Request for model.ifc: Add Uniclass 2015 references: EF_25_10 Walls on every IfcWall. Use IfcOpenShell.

First a look at what the model holds.

```python
import ifcopenshell

model = ifcopenshell.open("model.ifc")
print(model.schema)
print("classifications:", [c.Name for c in model.by_type("IfcClassification")])
for ifc_class in ("IfcDoor", "IfcRoof", "IfcStair", "IfcWall", "IfcWindow"):
    print(ifc_class, len(model.by_type(ifc_class)))
```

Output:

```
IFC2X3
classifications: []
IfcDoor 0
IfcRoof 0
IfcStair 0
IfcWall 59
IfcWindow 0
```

```python
import ifcopenshell
import ifcopenshell.api.classification

model = ifcopenshell.open("model.ifc")

# IFC2X3 requires Source and Edition and has no link from the project to the system.
system = model.create_entity("IfcClassification", Source="NBS", Edition="2015", Name="Uniclass 2015")

codes = {
    "IfcWall": ("EF_25_10", "Walls"),
}
for ifc_class, (code, name) in codes.items():
    products = model.by_type(ifc_class)
    ifcopenshell.api.classification.add_reference(
        model, products=products, classification=system, identification=code, name=name
    )
    print(code, len(products))

model.write("model_v2.ifc")
```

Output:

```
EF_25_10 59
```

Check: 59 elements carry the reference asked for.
